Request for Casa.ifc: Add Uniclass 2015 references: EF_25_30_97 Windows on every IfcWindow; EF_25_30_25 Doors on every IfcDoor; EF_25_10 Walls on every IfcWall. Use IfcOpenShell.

First a look at what the model holds.

```python
import ifcopenshell

model = ifcopenshell.open("Casa.ifc")
print(model.schema)
print("classifications:", [c.Name for c in model.by_type("IfcClassification")])
for ifc_class in ("IfcDoor", "IfcRoof", "IfcStair", "IfcWall", "IfcWindow"):
    print(ifc_class, len(model.by_type(ifc_class)))
```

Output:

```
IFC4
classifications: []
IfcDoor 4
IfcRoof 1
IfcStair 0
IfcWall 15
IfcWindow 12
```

```python
import ifcopenshell
import ifcopenshell.api.classification

model = ifcopenshell.open("Casa.ifc")

system = ifcopenshell.api.classification.add_classification(model, classification="Uniclass 2015")

codes = {
    "IfcWindow": ("EF_25_30_97", "Windows"),
    "IfcDoor": ("EF_25_30_25", "Doors"),
    "IfcWall": ("EF_25_10", "Walls"),
}
for ifc_class, (code, name) in codes.items():
    products = model.by_type(ifc_class)
    ifcopenshell.api.classification.add_reference(
        model, products=products, classification=system, identification=code, name=name
    )
    print(code, len(products))

model.write("Casa_rev.ifc")
```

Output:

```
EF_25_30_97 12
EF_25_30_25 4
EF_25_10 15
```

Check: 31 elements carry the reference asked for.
